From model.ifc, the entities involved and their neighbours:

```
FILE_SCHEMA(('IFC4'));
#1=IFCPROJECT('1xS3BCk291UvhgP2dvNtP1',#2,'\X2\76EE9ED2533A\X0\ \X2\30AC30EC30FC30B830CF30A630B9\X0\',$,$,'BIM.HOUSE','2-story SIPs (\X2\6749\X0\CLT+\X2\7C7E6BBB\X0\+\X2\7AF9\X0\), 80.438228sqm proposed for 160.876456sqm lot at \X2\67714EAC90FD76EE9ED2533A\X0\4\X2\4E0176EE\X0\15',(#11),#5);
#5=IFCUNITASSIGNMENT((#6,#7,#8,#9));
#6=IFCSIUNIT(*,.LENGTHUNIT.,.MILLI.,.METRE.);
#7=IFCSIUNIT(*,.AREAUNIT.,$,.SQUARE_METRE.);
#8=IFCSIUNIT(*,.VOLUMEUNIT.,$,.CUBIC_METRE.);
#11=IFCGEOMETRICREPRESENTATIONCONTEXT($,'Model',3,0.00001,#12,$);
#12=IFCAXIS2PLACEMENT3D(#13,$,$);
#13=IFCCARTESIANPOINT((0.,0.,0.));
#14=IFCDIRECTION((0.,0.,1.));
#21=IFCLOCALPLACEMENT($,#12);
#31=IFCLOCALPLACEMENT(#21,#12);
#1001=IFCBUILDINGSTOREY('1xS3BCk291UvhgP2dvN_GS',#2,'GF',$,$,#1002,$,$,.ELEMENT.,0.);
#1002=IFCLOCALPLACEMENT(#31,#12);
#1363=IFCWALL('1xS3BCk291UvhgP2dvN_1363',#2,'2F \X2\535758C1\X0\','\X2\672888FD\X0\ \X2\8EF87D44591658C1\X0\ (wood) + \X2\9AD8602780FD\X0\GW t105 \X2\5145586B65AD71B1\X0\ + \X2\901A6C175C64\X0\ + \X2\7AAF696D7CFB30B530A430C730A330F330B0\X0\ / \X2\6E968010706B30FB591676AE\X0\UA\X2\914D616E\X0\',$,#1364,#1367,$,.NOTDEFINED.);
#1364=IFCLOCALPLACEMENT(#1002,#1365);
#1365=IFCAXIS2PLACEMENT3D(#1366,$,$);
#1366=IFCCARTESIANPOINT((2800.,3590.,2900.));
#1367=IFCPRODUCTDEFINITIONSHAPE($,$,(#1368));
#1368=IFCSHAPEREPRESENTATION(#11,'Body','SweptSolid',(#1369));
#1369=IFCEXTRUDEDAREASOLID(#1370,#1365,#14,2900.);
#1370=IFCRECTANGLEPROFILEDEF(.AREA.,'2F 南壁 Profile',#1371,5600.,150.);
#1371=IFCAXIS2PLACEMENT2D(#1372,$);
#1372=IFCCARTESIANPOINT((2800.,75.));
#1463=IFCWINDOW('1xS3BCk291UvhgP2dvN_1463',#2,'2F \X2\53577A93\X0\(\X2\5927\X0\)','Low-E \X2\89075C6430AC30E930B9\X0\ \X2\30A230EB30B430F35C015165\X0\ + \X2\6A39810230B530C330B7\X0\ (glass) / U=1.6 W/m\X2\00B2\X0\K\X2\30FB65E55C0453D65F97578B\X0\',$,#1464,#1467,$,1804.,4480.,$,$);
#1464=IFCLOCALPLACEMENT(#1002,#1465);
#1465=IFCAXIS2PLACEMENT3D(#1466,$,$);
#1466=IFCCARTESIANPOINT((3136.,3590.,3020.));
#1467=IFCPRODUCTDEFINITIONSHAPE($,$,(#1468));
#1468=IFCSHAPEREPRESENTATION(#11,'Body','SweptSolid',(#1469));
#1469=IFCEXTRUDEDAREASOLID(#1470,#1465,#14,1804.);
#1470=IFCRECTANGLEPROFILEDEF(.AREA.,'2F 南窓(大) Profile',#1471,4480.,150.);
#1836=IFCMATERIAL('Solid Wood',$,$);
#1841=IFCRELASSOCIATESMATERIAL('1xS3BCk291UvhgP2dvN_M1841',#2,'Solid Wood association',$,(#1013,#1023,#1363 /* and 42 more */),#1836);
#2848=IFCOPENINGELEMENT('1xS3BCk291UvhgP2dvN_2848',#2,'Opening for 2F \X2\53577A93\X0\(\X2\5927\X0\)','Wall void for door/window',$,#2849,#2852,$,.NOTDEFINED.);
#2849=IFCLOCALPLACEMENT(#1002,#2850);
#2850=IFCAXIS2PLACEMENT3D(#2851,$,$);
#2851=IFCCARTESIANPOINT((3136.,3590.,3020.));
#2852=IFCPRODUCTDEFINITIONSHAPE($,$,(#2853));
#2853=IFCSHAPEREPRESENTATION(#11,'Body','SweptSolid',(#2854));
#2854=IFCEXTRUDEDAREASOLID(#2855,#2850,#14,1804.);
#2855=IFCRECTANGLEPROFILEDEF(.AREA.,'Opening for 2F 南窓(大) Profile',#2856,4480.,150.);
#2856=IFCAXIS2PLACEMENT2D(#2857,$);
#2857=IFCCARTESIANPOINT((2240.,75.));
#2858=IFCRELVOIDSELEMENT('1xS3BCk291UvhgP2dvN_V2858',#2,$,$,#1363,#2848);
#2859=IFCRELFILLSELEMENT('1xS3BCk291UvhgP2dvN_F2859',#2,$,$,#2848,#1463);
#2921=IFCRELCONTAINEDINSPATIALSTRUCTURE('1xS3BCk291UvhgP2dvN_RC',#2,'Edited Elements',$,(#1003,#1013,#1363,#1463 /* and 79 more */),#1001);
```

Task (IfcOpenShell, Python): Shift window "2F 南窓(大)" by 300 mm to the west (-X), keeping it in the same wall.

```python
import ifcopenshell
import ifcopenshell.api.geometry
import ifcopenshell.util.placement
import ifcopenshell.util.unit

model = ifcopenshell.open("model.ifc")
unit_scale = ifcopenshell.util.unit.calculate_unit_scale(model)

window = model.by_id(1463)
opening = window.FillsVoids[0].RelatingOpeningElement
wall = opening.VoidsElements[0].RelatingBuildingElement

wall_matrix = ifcopenshell.util.placement.get_local_placement(wall.ObjectPlacement)
shift = wall_matrix[:3, 0] * -0.3 / unit_scale
before = ifcopenshell.util.placement.get_local_placement(window.ObjectPlacement)[:3, 3].copy()

# The window is not placed relative to its opening, so move both.
for product in (opening, window):
    matrix = ifcopenshell.util.placement.get_local_placement(product.ObjectPlacement)
    matrix[:3, 3] += shift
    ifcopenshell.api.geometry.edit_object_placement(model, product=product, matrix=matrix, is_si=False)

after = ifcopenshell.util.placement.get_local_placement(window.ObjectPlacement)[:3, 3]
print("window moved by", (after - before).round(3) + 0.0)

model.write("model_edited.ifc")
```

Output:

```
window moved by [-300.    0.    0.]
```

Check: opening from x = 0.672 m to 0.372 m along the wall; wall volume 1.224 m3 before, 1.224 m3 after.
